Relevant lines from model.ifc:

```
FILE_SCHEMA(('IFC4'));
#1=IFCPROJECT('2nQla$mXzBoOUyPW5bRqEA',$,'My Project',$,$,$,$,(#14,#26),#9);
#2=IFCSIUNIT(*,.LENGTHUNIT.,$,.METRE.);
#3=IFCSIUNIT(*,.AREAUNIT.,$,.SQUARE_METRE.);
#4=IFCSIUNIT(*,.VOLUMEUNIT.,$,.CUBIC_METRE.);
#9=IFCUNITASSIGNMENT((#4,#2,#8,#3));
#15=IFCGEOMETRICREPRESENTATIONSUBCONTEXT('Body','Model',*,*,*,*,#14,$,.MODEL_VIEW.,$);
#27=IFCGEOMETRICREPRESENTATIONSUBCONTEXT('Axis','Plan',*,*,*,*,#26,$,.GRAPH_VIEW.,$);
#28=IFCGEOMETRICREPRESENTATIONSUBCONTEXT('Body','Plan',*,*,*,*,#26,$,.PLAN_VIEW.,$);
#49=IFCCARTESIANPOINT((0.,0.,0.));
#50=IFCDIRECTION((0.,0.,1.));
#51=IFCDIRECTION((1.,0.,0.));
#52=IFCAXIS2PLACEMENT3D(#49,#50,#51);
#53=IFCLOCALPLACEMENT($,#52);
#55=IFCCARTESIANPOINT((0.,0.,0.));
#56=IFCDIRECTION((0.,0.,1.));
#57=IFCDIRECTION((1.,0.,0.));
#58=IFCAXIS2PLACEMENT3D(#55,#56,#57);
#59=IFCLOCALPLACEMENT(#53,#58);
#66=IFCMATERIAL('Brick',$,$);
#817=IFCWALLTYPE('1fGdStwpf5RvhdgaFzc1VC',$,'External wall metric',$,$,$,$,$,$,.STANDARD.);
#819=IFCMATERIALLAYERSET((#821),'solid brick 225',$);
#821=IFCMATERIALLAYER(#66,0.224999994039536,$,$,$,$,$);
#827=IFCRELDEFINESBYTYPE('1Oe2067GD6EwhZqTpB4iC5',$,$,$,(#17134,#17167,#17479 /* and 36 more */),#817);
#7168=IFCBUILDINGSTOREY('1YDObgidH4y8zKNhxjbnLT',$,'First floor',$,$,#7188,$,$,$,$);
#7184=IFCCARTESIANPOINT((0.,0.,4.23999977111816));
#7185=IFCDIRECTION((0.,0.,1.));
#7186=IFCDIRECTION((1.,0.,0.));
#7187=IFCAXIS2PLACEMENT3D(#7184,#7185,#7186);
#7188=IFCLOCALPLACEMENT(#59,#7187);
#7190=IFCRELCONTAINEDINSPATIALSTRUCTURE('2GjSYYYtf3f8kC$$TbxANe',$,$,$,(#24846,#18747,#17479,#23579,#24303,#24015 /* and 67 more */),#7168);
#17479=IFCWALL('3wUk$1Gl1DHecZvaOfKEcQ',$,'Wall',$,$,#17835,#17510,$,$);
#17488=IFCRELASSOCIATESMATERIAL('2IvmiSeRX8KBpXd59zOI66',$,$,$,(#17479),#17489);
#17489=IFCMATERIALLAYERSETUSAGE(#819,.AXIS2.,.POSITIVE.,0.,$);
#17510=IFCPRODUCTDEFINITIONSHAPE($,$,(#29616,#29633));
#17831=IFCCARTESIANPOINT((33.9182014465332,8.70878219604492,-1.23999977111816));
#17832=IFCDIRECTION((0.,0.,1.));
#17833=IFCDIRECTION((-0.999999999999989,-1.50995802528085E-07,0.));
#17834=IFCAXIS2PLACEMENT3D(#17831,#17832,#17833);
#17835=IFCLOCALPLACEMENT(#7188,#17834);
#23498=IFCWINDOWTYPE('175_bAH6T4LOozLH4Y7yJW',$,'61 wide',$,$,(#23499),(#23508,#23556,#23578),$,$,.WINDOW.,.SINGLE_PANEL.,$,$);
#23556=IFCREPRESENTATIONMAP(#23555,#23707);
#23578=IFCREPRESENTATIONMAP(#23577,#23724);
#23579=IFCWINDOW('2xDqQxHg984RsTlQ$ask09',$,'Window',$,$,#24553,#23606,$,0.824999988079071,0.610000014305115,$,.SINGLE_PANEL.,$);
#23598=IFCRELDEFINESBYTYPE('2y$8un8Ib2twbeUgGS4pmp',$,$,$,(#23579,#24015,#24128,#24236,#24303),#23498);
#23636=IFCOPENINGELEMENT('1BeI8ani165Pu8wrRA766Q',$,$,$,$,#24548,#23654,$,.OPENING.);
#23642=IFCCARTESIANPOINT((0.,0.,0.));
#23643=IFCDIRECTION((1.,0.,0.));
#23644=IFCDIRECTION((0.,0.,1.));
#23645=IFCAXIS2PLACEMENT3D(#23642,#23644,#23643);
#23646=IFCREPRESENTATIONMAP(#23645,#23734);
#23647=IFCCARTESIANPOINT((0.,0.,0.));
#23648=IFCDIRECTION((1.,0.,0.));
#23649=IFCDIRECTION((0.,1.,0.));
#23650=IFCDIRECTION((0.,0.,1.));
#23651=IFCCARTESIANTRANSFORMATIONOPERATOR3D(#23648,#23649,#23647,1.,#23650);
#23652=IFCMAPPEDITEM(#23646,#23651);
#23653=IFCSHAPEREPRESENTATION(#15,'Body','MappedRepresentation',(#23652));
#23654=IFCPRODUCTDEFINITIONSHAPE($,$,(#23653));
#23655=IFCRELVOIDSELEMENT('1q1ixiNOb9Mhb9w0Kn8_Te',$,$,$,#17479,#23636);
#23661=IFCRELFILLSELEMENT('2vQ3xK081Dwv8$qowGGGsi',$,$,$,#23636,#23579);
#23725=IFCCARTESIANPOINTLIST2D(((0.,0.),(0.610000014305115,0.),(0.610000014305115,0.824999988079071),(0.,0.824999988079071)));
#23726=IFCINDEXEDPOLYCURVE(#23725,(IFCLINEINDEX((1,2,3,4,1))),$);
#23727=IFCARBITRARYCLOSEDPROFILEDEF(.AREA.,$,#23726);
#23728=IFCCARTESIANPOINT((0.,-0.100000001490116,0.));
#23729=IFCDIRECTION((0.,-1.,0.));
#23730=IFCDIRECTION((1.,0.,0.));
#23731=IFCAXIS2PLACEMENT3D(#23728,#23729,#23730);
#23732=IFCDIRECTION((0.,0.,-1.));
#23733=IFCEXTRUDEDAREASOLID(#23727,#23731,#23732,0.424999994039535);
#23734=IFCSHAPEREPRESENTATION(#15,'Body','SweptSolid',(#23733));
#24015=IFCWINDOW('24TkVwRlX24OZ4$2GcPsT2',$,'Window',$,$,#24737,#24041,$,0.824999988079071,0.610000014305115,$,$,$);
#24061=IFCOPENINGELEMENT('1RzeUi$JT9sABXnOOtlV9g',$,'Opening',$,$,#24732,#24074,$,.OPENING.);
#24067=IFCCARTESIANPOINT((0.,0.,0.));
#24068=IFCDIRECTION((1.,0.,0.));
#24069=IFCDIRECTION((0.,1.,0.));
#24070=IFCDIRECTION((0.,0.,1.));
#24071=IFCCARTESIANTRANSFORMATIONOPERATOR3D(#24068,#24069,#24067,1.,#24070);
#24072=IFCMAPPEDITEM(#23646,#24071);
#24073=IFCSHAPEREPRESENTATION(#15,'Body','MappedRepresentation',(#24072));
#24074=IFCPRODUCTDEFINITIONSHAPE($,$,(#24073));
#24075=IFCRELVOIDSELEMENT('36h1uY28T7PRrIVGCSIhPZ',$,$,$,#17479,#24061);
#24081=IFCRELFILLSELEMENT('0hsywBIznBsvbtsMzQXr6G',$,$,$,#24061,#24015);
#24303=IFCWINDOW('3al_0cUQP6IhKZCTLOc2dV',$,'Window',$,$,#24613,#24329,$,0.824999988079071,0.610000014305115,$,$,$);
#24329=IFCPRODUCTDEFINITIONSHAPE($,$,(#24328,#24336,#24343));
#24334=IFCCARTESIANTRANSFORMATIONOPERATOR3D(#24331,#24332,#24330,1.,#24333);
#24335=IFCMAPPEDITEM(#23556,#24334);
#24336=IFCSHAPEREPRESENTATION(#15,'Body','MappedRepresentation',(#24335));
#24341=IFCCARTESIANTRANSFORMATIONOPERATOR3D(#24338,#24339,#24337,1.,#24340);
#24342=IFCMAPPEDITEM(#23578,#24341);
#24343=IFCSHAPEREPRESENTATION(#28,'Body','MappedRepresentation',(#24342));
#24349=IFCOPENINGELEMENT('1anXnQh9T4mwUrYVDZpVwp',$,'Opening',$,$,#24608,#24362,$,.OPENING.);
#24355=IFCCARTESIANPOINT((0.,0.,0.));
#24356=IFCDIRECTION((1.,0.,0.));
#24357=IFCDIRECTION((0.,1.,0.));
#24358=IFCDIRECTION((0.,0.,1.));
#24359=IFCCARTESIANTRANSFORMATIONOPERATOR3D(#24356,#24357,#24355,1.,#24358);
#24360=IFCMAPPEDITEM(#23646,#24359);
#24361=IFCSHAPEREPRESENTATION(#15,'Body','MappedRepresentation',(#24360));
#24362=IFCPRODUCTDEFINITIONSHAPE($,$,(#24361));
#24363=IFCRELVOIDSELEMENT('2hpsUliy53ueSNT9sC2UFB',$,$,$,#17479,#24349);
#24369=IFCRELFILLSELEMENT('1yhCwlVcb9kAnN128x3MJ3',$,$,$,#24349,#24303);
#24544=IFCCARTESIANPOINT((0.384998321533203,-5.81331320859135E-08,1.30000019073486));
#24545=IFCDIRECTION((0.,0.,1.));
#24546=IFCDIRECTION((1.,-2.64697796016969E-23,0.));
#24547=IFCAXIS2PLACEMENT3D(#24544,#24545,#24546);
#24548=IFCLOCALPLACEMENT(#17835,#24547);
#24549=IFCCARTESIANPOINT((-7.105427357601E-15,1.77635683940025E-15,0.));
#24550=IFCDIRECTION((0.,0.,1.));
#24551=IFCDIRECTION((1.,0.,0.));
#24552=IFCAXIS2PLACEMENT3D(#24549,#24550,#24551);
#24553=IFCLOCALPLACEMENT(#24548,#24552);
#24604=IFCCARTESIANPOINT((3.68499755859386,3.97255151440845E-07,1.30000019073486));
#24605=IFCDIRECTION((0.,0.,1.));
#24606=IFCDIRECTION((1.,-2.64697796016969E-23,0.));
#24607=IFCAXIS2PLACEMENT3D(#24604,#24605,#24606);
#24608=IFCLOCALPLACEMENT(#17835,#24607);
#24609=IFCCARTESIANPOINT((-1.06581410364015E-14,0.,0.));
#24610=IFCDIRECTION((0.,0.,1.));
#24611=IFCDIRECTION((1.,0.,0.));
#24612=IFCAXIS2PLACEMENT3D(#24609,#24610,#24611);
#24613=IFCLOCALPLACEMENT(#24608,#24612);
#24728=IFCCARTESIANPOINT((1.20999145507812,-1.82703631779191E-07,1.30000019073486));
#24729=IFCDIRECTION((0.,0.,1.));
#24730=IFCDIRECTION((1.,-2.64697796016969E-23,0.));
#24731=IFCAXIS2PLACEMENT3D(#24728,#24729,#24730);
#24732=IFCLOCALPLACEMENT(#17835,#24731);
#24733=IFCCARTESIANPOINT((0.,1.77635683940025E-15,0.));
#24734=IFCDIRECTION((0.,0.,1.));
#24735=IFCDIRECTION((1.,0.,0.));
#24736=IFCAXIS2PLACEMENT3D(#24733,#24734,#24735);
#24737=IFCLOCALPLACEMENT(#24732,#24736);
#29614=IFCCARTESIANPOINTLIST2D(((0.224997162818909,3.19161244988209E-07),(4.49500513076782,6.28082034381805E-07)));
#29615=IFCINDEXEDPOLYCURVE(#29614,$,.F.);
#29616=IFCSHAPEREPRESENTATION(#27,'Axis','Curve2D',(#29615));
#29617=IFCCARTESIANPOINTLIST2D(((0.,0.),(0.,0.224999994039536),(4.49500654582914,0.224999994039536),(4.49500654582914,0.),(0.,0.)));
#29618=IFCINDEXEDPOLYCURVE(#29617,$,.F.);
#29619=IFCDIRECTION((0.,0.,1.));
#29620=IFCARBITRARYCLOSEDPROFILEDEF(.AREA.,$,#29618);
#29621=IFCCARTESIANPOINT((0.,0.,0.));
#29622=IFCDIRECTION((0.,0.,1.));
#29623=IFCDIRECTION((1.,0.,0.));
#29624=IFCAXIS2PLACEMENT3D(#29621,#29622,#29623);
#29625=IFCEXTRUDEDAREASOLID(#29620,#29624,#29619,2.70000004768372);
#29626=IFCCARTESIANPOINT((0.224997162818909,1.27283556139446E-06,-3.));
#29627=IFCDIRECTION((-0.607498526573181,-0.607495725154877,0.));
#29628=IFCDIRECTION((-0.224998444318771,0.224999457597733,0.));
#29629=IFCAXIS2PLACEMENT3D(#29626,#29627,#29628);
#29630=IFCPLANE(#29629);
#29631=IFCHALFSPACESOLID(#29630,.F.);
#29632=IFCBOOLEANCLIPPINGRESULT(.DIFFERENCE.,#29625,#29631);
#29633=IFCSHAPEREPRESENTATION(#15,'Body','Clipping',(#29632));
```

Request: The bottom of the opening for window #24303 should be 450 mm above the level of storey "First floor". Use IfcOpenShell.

```python
import numpy as np
import ifcopenshell
import ifcopenshell.api.geometry
import ifcopenshell.geom
import ifcopenshell.util.element
import ifcopenshell.util.placement
import ifcopenshell.util.shape
import ifcopenshell.util.unit

model = ifcopenshell.open("model.ifc")
unit_scale = ifcopenshell.util.unit.calculate_unit_scale(model)

window = model.by_guid("3al_0cUQP6IhKZCTLOc2dV")
opening = window.FillsVoids[0].RelatingOpeningElement
storey = ifcopenshell.util.element.get_container(window, ifc_class="IfcBuildingStorey")
level = ifcopenshell.util.placement.get_local_placement(storey.ObjectPlacement)[2, 3]

# The opening's origin need not be at the sill, so measure its lowest point.
shape = ifcopenshell.geom.create_shape(ifcopenshell.geom.settings(), opening)
bottom = ifcopenshell.util.shape.get_shape_bottom_elevation(shape, shape.geometry) / unit_scale
dz = level + 0.45 - bottom

shift = np.array([0.0, 0.0, dz])
# The window is placed relative to its opening, so it follows when the opening moves.
matrix = ifcopenshell.util.placement.get_local_placement(opening.ObjectPlacement)
matrix[:3, 3] += shift
ifcopenshell.api.geometry.edit_object_placement(
    model, product=opening, matrix=matrix, is_si=False, should_transform_children=True
)

print(f"moved by {dz * unit_scale:+.3f} m")

model.write("model-out.ifc")
```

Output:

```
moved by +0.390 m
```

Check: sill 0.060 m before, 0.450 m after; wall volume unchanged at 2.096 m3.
